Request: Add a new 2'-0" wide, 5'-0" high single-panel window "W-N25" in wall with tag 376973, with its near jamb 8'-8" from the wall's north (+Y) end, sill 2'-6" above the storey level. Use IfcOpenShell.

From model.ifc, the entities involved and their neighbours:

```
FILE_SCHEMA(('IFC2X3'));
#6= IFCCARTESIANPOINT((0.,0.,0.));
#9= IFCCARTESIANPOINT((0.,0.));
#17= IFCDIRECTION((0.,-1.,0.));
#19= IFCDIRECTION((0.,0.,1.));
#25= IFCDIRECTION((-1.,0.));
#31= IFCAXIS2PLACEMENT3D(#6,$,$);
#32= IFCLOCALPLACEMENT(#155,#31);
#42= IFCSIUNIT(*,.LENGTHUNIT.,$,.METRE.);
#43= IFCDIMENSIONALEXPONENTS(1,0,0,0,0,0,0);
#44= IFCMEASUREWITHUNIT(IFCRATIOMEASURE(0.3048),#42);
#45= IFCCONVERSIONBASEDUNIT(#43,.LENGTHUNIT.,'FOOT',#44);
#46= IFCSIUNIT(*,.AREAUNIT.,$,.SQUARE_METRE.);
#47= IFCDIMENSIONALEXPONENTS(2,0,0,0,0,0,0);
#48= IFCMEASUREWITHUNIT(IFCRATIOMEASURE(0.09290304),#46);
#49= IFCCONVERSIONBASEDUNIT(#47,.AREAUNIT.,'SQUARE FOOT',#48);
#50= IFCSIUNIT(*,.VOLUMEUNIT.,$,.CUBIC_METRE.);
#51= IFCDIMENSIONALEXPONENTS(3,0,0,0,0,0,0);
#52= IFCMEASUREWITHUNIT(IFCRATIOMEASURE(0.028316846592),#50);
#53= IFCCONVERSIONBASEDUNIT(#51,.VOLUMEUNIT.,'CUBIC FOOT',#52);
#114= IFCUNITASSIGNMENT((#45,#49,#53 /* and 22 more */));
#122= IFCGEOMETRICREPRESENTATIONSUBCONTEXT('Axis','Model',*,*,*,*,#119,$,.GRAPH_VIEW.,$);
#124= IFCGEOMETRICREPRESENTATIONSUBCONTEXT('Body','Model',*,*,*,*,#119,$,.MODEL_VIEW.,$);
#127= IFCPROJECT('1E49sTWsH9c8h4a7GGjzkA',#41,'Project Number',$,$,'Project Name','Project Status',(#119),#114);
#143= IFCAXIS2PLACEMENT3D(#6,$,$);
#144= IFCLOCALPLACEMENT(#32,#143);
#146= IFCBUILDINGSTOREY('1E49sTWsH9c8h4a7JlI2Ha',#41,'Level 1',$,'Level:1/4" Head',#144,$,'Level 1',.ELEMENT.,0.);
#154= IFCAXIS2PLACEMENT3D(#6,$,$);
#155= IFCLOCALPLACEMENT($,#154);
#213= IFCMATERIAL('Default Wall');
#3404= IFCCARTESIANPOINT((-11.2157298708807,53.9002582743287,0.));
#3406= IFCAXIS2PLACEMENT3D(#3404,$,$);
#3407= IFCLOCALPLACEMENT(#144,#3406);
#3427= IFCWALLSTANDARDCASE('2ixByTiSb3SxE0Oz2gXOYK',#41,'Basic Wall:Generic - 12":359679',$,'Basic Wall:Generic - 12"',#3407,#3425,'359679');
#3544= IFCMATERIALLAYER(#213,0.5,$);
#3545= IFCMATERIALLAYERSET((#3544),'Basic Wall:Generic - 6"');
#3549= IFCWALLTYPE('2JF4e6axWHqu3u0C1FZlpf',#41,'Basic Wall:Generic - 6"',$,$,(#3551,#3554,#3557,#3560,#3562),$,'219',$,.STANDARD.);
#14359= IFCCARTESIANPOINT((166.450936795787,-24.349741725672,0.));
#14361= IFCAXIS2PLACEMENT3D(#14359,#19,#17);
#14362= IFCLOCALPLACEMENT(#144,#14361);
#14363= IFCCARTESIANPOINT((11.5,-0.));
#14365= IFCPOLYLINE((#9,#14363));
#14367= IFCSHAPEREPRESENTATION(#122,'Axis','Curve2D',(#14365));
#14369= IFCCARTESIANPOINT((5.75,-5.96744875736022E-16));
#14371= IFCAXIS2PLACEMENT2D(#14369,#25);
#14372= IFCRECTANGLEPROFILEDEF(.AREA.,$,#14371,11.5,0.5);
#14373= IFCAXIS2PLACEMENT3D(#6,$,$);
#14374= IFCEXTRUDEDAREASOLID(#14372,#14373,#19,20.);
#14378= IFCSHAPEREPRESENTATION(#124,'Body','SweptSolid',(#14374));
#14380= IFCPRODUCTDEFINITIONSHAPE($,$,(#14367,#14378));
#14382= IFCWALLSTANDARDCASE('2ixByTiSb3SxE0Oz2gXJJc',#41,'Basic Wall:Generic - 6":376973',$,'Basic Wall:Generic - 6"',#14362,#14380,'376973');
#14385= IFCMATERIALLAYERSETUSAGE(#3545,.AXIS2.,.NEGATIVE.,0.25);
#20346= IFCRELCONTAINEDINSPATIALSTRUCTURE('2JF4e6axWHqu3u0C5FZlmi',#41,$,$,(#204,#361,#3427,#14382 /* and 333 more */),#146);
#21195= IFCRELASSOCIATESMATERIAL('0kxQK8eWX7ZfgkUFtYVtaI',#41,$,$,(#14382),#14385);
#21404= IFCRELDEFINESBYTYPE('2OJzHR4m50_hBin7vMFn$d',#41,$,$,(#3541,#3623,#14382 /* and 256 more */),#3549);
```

```python
import numpy as np
import ifcopenshell
import ifcopenshell.api.feature
import ifcopenshell.api.geometry
import ifcopenshell.api.root
import ifcopenshell.api.spatial
import ifcopenshell.api.type
import ifcopenshell.geom
import ifcopenshell.util.element
import ifcopenshell.util.placement
import ifcopenshell.util.representation
import ifcopenshell.util.shape
import ifcopenshell.util.unit

model = ifcopenshell.open("model.ifc")
unit_scale = ifcopenshell.util.unit.calculate_unit_scale(model)
settings = ifcopenshell.geom.settings()


def volume(element):
    """Net volume in cubic metres, openings subtracted."""
    shape = ifcopenshell.geom.create_shape(settings, element)
    return ifcopenshell.util.shape.get_volume(shape.geometry)


wall = model.by_id(14382)
storey = ifcopenshell.util.element.get_container(wall, ifc_class="IfcBuildingStorey")
context = ifcopenshell.util.representation.get_context(model, "Model", "Body", "MODEL_VIEW")
before = volume(wall)

width, height, from_end, sill = 0.6096, 1.524, 2.6416, 0.762  # metres

# The wall runs along its own X axis, and the end named is its -X end.
wall_shape = ifcopenshell.geom.create_shape(settings, wall)
x, y, z = ifcopenshell.util.shape.get_vertices(wall_shape.geometry).T
start = x.min() + from_end
face, thickness = float(y.min()), float(y.max() - y.min())
wall_matrix = ifcopenshell.util.placement.get_local_placement(wall.ObjectPlacement)
level = ifcopenshell.util.placement.get_local_placement(storey.ObjectPlacement)[2, 3]


def in_wall(x, y):
    """Placement at x, y metres in the wall's axes, at sill height."""
    matrix = wall_matrix.copy()
    matrix[:, 3] = wall_matrix @ np.array([x / unit_scale, y / unit_scale, 0.0, 1.0])
    matrix[2, 3] = level + sill / unit_scale
    return matrix


# Opening: a box that overshoots both wall faces by 50 mm.
opening = ifcopenshell.api.root.create_entity(model, ifc_class="IfcOpeningElement")
box = ifcopenshell.api.geometry.add_wall_representation(
    model, context=context, length=width, height=height, thickness=thickness + 0.1
)
ifcopenshell.api.geometry.assign_representation(model, product=opening, representation=box)
ifcopenshell.api.geometry.edit_object_placement(model, product=opening, matrix=in_wall(start, face - 0.05), is_si=False)
ifcopenshell.api.feature.add_feature(model, feature=opening, element=wall)

window = ifcopenshell.api.root.create_entity(model, ifc_class="IfcWindow", name="W-N25")
window.OverallWidth, window.OverallHeight = width / unit_scale, height / unit_scale
body = ifcopenshell.api.geometry.add_window_representation(
    model,
    context=context,
    overall_width=window.OverallWidth,
    overall_height=window.OverallHeight,
    partition_type="SINGLE_PANEL",
)
ifcopenshell.api.geometry.assign_representation(model, product=window, representation=body)
ifcopenshell.api.spatial.assign_container(model, products=[window], relating_structure=storey)
fills = ifcopenshell.api.feature.add_filling(model, opening=opening, element=window)
fills.OwnerHistory = window.OwnerHistory  # required in IFC2X3

# IFC2X3 keeps the operation on the window style.
style = ifcopenshell.api.root.create_entity(model, ifc_class="IfcWindowStyle", name="W-N25")
style.OperationType, style.ConstructionType = "SINGLE_PANEL", "NOTDEFINED"
style.ParameterTakesPrecedence = style.Sizeable = False
ifcopenshell.api.type.assign_type(model, related_objects=[window], relating_type=style)

# Centre the window in the wall's thickness.
ifcopenshell.api.geometry.edit_object_placement(model, product=window, matrix=in_wall(start, face), is_si=False)
window_shape = ifcopenshell.geom.create_shape(settings, window)
depth = ifcopenshell.util.shape.get_vertices(window_shape.geometry)[:, 1]
offset = face + thickness / 2 - (depth.min() + depth.max()) / 2
ifcopenshell.api.geometry.edit_object_placement(model, product=window, matrix=in_wall(start, offset), is_si=False)

after = volume(wall)

print(f"wall volume {before:.3f} -> {after:.3f} m3")

model.write("model_v2.ifc")
```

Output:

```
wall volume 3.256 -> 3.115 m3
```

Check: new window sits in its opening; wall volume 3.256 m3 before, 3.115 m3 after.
